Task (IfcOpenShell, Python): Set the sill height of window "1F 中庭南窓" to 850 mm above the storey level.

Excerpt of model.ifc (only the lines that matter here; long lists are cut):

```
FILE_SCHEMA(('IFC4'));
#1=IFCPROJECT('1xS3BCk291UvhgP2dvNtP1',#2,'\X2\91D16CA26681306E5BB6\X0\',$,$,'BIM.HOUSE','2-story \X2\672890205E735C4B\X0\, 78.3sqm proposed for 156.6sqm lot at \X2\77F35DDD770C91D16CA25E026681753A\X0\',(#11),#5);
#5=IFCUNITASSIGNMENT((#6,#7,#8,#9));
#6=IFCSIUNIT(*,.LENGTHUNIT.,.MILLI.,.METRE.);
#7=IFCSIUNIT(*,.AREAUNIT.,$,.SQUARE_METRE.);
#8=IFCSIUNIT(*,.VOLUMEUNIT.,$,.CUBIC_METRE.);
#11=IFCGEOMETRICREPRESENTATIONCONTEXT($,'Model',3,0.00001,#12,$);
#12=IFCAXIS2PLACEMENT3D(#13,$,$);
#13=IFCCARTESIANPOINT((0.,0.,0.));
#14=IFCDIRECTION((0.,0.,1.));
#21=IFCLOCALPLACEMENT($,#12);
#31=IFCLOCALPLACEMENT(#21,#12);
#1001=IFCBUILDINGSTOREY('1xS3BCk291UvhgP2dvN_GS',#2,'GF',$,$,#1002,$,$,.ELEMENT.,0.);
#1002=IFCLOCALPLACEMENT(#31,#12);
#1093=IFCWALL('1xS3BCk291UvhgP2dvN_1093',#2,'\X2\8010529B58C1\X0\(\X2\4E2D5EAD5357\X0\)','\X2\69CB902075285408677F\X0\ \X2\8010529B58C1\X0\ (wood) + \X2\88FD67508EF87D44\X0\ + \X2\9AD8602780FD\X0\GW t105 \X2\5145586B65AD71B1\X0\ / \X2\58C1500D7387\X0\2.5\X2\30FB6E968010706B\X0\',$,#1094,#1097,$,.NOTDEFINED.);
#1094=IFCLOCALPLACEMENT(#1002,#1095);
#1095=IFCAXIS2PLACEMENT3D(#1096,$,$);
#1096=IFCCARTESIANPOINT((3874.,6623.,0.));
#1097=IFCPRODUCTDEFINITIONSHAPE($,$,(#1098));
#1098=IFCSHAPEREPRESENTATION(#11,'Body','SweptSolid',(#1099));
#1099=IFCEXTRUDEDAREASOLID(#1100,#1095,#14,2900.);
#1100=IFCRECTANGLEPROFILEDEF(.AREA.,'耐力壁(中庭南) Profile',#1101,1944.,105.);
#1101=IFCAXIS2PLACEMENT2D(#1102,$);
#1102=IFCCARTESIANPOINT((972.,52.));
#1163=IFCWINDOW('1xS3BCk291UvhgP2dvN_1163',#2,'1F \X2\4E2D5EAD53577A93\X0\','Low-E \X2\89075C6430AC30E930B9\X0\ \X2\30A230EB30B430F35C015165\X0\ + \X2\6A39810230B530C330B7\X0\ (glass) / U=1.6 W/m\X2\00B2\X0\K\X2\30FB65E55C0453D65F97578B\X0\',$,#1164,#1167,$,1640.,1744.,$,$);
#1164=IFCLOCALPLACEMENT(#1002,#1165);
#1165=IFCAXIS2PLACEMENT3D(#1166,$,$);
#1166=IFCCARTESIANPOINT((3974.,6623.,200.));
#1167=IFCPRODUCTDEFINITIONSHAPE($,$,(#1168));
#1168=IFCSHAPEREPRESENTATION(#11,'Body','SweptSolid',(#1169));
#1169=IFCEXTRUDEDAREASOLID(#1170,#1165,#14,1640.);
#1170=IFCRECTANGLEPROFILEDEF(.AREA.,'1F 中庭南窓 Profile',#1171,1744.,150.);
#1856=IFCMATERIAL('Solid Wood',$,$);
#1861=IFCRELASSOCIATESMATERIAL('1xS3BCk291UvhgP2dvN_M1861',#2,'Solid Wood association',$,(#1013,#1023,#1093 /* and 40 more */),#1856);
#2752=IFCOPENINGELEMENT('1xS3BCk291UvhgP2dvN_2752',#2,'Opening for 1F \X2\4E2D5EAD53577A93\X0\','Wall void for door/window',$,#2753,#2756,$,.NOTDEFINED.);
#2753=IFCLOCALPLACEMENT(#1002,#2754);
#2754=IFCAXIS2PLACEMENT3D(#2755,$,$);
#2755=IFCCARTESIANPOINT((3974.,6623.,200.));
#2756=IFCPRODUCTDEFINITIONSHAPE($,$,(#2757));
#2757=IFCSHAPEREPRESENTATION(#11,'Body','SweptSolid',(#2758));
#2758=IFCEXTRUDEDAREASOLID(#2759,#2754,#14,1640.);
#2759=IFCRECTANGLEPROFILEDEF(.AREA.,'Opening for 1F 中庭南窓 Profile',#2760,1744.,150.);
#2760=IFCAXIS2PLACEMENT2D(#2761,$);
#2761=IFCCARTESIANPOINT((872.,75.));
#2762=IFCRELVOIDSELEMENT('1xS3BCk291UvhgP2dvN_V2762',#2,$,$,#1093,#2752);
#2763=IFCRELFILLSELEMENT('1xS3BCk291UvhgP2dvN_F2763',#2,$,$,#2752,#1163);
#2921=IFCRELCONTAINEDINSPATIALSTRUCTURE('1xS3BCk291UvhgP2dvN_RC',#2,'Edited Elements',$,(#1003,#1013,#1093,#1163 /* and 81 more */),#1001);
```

```python
import numpy as np
import ifcopenshell
import ifcopenshell.api.geometry
import ifcopenshell.geom
import ifcopenshell.util.element
import ifcopenshell.util.placement
import ifcopenshell.util.shape
import ifcopenshell.util.unit

model = ifcopenshell.open("model.ifc")
unit_scale = ifcopenshell.util.unit.calculate_unit_scale(model)

window = model.by_guid("1xS3BCk291UvhgP2dvN_1163")
opening = window.FillsVoids[0].RelatingOpeningElement
storey = ifcopenshell.util.element.get_container(window, ifc_class="IfcBuildingStorey")
level = ifcopenshell.util.placement.get_local_placement(storey.ObjectPlacement)[2, 3]

# The opening's origin need not be at the sill, so measure its lowest point.
shape = ifcopenshell.geom.create_shape(ifcopenshell.geom.settings(), opening)
bottom = ifcopenshell.util.shape.get_shape_bottom_elevation(shape, shape.geometry) / unit_scale
dz = level + 850.0 - bottom

shift = np.array([0.0, 0.0, dz])
# The window is not placed relative to its opening, so move both.
for product in (opening, window):
    matrix = ifcopenshell.util.placement.get_local_placement(product.ObjectPlacement)
    matrix[:3, 3] += shift
    ifcopenshell.api.geometry.edit_object_placement(model, product=product, matrix=matrix, is_si=False)

print(f"moved by {dz * unit_scale:+.3f} m")

model.write("model-out.ifc")
```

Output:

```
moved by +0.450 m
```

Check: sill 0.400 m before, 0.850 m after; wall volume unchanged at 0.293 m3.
